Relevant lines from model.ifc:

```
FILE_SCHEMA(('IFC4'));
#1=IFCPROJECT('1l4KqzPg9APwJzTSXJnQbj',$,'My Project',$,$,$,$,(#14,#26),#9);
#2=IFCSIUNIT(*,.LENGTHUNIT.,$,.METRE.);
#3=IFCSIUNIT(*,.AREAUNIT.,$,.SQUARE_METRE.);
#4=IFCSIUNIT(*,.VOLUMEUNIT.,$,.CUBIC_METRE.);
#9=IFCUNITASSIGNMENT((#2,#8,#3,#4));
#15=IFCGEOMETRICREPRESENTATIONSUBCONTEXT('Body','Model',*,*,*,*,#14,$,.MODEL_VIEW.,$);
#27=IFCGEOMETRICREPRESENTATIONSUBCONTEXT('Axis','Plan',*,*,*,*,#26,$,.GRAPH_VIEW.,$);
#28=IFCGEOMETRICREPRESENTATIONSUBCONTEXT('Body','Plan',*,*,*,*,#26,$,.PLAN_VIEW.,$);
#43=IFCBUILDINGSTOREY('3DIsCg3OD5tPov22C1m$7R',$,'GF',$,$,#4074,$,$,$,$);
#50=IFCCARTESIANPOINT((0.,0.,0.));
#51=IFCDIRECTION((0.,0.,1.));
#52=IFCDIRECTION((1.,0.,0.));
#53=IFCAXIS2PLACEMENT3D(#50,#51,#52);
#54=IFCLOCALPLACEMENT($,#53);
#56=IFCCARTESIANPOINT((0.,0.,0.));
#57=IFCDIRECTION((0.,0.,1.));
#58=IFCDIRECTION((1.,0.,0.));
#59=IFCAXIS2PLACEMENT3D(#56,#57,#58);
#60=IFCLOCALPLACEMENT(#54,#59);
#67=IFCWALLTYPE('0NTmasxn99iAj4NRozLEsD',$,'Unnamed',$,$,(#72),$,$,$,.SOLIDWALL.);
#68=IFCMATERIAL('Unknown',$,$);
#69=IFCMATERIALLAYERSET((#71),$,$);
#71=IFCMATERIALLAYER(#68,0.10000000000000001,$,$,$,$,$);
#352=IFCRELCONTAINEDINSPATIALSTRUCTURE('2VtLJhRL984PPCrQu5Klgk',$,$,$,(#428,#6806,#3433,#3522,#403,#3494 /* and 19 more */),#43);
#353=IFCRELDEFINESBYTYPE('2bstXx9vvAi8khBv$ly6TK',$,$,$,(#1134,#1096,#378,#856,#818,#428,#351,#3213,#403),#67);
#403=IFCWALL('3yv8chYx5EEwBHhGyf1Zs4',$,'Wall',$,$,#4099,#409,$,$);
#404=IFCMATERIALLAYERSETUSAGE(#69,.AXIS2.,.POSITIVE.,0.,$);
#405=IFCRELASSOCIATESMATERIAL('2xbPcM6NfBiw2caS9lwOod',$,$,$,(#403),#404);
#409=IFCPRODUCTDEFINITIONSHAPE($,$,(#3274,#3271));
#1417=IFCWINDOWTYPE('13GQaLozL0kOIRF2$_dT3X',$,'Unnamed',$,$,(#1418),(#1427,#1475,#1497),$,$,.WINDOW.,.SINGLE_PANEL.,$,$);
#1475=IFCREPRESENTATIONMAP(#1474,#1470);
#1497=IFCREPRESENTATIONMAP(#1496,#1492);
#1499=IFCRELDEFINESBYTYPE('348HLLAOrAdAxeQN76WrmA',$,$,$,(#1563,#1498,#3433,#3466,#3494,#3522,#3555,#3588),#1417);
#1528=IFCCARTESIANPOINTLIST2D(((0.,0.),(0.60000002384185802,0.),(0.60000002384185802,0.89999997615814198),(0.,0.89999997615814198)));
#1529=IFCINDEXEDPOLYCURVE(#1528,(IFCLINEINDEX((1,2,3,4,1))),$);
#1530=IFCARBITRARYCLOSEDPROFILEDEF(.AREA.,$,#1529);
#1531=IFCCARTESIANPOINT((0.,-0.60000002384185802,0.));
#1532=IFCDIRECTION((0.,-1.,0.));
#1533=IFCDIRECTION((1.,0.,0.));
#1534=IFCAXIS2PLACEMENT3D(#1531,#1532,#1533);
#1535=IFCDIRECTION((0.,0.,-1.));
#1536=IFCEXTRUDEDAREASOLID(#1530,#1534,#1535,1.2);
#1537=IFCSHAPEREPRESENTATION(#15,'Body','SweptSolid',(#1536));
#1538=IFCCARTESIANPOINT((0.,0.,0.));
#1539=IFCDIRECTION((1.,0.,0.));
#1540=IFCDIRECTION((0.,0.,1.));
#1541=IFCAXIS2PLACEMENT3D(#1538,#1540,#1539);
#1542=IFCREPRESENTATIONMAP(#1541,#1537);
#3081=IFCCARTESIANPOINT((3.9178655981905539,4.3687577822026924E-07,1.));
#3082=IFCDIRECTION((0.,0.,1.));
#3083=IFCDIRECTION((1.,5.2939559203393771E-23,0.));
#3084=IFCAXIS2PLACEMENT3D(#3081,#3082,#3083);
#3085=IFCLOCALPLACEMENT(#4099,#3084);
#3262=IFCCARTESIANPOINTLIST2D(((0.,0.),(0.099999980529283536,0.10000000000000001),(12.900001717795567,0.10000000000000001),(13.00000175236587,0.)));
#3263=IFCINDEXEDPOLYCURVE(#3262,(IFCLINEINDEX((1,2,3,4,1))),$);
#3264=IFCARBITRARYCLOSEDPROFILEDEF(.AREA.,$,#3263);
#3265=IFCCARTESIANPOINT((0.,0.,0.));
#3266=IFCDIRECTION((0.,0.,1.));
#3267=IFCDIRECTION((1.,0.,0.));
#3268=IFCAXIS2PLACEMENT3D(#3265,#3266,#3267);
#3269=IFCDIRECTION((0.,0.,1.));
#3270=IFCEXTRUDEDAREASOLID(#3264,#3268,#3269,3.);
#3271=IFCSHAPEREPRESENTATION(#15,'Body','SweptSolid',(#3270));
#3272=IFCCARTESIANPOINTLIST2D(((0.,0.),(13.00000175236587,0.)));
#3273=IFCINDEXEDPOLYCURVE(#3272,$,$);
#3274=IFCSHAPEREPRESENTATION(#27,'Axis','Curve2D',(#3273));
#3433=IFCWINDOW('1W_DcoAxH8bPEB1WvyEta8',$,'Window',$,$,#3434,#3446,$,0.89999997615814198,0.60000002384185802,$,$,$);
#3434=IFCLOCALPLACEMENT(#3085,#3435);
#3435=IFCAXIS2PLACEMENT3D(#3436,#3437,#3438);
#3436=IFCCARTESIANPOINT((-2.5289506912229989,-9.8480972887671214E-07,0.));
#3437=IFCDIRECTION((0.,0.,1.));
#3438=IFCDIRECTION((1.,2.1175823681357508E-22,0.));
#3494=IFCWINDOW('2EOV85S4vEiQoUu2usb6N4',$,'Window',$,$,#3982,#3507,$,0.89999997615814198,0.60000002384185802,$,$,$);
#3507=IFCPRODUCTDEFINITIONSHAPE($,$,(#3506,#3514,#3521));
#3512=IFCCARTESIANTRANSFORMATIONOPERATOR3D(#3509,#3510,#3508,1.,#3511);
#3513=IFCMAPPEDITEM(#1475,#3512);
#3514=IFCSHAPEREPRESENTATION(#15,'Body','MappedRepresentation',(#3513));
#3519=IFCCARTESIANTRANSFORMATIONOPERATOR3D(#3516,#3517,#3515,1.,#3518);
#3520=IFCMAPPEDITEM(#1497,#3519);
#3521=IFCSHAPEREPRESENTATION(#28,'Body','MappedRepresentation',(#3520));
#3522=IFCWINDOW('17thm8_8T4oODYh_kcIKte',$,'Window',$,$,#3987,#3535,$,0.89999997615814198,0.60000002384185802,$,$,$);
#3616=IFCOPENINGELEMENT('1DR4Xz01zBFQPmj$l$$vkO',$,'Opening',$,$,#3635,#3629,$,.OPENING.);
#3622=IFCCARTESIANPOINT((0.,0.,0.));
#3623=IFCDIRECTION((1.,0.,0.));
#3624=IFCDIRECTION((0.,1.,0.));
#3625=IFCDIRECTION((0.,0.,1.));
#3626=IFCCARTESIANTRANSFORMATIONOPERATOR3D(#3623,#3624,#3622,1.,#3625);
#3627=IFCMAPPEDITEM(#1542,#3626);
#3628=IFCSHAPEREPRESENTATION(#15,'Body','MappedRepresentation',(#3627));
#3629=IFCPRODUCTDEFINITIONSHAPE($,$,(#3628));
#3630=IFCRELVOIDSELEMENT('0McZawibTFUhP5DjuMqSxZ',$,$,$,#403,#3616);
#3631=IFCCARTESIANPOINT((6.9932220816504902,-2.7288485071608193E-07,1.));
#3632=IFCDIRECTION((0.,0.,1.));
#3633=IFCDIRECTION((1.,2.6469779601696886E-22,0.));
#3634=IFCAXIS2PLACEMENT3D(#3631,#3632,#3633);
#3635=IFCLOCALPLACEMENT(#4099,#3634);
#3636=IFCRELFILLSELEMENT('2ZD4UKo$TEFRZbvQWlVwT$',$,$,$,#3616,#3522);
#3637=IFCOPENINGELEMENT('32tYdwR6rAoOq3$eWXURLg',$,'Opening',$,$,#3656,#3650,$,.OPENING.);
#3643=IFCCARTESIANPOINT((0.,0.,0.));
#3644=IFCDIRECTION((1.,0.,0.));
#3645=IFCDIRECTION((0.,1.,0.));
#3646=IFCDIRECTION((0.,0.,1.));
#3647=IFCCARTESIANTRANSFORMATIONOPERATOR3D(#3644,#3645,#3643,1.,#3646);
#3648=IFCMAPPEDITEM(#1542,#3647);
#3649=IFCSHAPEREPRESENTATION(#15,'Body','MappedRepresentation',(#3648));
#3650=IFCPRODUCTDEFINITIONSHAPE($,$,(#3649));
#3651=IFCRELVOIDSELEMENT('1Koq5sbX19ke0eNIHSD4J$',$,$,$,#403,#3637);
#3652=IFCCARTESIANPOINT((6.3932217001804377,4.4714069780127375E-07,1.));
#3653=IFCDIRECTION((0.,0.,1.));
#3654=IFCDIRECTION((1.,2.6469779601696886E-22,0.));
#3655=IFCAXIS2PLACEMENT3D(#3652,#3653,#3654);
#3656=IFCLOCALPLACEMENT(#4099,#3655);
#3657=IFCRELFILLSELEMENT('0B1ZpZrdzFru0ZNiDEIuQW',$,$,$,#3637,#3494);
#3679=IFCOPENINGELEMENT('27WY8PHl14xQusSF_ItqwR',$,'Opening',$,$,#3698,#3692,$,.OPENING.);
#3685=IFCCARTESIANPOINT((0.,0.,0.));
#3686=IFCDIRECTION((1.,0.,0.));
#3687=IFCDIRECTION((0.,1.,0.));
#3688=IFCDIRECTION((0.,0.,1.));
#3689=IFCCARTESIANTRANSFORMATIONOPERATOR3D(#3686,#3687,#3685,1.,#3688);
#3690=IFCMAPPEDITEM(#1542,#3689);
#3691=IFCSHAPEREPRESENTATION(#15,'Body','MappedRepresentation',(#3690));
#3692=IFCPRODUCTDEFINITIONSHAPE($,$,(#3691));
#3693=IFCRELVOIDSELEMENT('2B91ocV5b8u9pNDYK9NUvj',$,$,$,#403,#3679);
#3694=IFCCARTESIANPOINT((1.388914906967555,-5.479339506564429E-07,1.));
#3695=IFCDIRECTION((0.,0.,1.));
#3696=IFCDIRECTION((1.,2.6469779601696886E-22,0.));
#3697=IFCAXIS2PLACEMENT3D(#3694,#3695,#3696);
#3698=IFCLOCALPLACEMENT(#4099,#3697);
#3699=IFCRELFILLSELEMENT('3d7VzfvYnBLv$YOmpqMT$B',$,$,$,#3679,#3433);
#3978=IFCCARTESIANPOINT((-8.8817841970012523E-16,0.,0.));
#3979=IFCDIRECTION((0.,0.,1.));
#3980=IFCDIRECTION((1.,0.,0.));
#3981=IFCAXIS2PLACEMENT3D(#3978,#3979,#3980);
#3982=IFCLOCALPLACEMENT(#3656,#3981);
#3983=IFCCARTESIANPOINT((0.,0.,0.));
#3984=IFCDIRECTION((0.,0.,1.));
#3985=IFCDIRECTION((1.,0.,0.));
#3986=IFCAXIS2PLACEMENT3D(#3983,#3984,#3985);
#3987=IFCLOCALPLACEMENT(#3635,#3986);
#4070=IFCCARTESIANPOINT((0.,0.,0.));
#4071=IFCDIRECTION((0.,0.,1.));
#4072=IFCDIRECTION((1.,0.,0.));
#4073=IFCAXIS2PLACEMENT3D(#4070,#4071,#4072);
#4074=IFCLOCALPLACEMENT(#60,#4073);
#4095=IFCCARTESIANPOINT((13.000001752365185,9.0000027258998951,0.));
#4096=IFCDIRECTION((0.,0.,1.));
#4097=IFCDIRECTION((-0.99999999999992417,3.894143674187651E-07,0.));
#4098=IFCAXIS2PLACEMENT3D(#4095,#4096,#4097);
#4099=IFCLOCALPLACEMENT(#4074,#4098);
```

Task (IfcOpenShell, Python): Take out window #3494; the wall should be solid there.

```python
import ifcopenshell
import ifcopenshell.api.feature
import ifcopenshell.api.root
import ifcopenshell.geom
import ifcopenshell.util.shape

model = ifcopenshell.open("model.ifc")
settings = ifcopenshell.geom.settings()


def volume(element):
    """Net volume in cubic metres, openings subtracted."""
    shape = ifcopenshell.geom.create_shape(settings, element)
    return ifcopenshell.util.shape.get_volume(shape.geometry)


window = model.by_id(3494)
opening = window.FillsVoids[0].RelatingOpeningElement
wall = opening.VoidsElements[0].RelatingBuildingElement
before = volume(wall)

ifcopenshell.api.root.remove_product(model, product=window)
ifcopenshell.api.feature.remove_feature(model, feature=opening)

after = volume(wall)

print(f"wall volume {before:.3f} -> {after:.3f} m3")

model.write("model-out.ifc")
```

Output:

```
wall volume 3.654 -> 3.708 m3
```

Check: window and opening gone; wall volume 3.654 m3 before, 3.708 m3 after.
